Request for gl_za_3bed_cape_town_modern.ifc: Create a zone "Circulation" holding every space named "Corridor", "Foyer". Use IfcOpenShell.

First a look at what the model holds.

```python
import ifcopenshell

model = ifcopenshell.open("gl_za_3bed_cape_town_modern.ifc")
print(model.schema)
seen = {}
for space in model.by_type("IfcSpace"):
    seen[space.LongName] = seen.get(space.LongName, 0) + 1
for name, count in sorted(seen.items(), key=str):
    print(count, "x", name)
print("zones:", [z.Name for z in model.by_type("IfcZone")][:20])
```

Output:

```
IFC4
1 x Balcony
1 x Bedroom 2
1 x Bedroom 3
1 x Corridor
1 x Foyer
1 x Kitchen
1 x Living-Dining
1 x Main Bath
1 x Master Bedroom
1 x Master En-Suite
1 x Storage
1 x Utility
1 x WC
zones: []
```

```python
import ifcopenshell
import ifcopenshell.api.group
import ifcopenshell.api.root

model = ifcopenshell.open("gl_za_3bed_cape_town_modern.ifc")

names = {"Corridor", "Foyer"}
spaces = [s for s in model.by_type("IfcSpace") if s.LongName in names]

zone = ifcopenshell.api.root.create_entity(model, ifc_class="IfcZone", name="Circulation")
ifcopenshell.api.group.assign_group(model, products=spaces, group=zone)
print(len(spaces), "spaces in", zone.Name)

model.write("gl_za_3bed_cape_town_modern_edited.ifc")
```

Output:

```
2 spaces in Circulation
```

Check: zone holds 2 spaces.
